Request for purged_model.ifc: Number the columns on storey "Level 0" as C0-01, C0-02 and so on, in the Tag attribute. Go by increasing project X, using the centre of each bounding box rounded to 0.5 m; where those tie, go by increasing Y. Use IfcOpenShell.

First a look at what the model holds.

```python
import ifcopenshell
import ifcopenshell.util.element
import ifcopenshell.util.placement

model = ifcopenshell.open("purged_model.ifc")
print(model.schema)
storey = next(s for s in model.by_type("IfcBuildingStorey") if s.Name == "Level 0")
columns = [e for e in ifcopenshell.util.element.get_decomposition(storey) if e.is_a("IfcColumn")]
for e in sorted(columns, key=lambda e: e.id()):
    origin = ifcopenshell.util.placement.get_local_placement(e.ObjectPlacement)[:3, 3]
    print(e.id(), e.Tag, e.Name, origin.round(2) + 0.0, sep=" | ")
```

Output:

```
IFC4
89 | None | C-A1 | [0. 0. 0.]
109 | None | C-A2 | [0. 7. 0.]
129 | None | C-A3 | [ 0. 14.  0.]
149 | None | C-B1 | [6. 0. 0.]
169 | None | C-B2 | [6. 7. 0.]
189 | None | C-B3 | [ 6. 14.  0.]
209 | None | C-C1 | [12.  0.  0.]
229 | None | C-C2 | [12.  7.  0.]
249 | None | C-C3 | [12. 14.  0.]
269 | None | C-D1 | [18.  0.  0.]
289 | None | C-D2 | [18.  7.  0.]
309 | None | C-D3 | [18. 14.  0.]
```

```python
import ifcopenshell
import ifcopenshell.geom
import ifcopenshell.util.element
import ifcopenshell.util.shape

model = ifcopenshell.open("purged_model.ifc")
settings = ifcopenshell.geom.settings()
settings.set("use-world-coords", True)


def centre(element):
    shape = ifcopenshell.geom.create_shape(settings, element)
    return ifcopenshell.util.shape.get_bbox_centroid(shape.geometry)


storey = next(s for s in model.by_type("IfcBuildingStorey") if s.Name == "Level 0")
columns = [e for e in ifcopenshell.util.element.get_decomposition(storey) if e.is_a("IfcColumn")]

# Insertion points can sit at a corner or the storey origin, so sort by the geometry (in metres).
centres = {e: centre(e) for e in columns}
columns.sort(key=lambda e: (round(centres[e][0] / 0.5), centres[e][1]))

for i, e in enumerate(columns, start=1):
    number = f"C0-{i:02d}"
    e.Tag = number
    print(e.id(), number)

model.write("purged_model_rev.ifc")
```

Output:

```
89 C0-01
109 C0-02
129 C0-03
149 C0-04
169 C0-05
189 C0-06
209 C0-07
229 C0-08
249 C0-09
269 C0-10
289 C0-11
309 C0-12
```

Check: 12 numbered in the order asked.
